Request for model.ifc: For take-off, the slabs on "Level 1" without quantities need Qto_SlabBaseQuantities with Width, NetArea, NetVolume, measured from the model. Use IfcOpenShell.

First a look at what the model holds.

```python
import ifcopenshell
import ifcopenshell.util.element
import ifcopenshell.util.unit

model = ifcopenshell.open("model.ifc")
print(model.schema)
for unit_type in ("LENGTHUNIT", "AREAUNIT", "VOLUMEUNIT"):
    print(unit_type, ifcopenshell.util.unit.calculate_unit_scale(model, unit_type))
storey = next(s for s in model.by_type("IfcBuildingStorey") if s.Name == "Level 1")
slabs = [e for e in ifcopenshell.util.element.get_decomposition(storey) if e.is_a("IfcSlab")]
for e in sorted(slabs, key=lambda e: e.id()):
    print(e.id(), e.is_a(), e.Name, list(ifcopenshell.util.element.get_psets(e, qtos_only=True)), sep=" | ")
```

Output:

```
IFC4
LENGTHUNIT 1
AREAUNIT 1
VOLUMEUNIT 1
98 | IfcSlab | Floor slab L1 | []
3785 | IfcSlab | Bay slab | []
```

```python
import ifcopenshell
import ifcopenshell.api.pset
import ifcopenshell.geom
import ifcopenshell.util.element
import ifcopenshell.util.shape
import ifcopenshell.util.unit

model = ifcopenshell.open("model.ifc")
unit_scale = ifcopenshell.util.unit.calculate_unit_scale(model)
area_scale = ifcopenshell.util.unit.calculate_unit_scale(model, "AREAUNIT")
volume_scale = ifcopenshell.util.unit.calculate_unit_scale(model, "VOLUMEUNIT")
settings = ifcopenshell.geom.settings()

storey = next(s for s in model.by_type("IfcBuildingStorey") if s.Name == "Level 1")
slabs = [e for e in ifcopenshell.util.element.get_decomposition(storey) if e.is_a("IfcSlab")]

for e in sorted(slabs, key=lambda e: e.id()):
    if ifcopenshell.util.element.get_psets(e, qtos_only=True, should_inherit=False):
        continue
    # Geometry comes back in metres, in the element's own axes.
    shape = ifcopenshell.geom.create_shape(settings, e)
    values = {
        "Width": ifcopenshell.util.shape.get_z(shape.geometry) / unit_scale,
        "NetArea": ifcopenshell.util.shape.get_footprint_area(shape.geometry) / area_scale,
        "NetVolume": ifcopenshell.util.shape.get_volume(shape.geometry) / volume_scale,
    }
    qto = ifcopenshell.api.pset.add_qto(model, product=e, name="Qto_SlabBaseQuantities")
    ifcopenshell.api.pset.edit_qto(model, qto=qto, properties=values)
    print(e.id(), {k: round(v, 3) for k, v in values.items()})

model.write("model_rev.ifc")
```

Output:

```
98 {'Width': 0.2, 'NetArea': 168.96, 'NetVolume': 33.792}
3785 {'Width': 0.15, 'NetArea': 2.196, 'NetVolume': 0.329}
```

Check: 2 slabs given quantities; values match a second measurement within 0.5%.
